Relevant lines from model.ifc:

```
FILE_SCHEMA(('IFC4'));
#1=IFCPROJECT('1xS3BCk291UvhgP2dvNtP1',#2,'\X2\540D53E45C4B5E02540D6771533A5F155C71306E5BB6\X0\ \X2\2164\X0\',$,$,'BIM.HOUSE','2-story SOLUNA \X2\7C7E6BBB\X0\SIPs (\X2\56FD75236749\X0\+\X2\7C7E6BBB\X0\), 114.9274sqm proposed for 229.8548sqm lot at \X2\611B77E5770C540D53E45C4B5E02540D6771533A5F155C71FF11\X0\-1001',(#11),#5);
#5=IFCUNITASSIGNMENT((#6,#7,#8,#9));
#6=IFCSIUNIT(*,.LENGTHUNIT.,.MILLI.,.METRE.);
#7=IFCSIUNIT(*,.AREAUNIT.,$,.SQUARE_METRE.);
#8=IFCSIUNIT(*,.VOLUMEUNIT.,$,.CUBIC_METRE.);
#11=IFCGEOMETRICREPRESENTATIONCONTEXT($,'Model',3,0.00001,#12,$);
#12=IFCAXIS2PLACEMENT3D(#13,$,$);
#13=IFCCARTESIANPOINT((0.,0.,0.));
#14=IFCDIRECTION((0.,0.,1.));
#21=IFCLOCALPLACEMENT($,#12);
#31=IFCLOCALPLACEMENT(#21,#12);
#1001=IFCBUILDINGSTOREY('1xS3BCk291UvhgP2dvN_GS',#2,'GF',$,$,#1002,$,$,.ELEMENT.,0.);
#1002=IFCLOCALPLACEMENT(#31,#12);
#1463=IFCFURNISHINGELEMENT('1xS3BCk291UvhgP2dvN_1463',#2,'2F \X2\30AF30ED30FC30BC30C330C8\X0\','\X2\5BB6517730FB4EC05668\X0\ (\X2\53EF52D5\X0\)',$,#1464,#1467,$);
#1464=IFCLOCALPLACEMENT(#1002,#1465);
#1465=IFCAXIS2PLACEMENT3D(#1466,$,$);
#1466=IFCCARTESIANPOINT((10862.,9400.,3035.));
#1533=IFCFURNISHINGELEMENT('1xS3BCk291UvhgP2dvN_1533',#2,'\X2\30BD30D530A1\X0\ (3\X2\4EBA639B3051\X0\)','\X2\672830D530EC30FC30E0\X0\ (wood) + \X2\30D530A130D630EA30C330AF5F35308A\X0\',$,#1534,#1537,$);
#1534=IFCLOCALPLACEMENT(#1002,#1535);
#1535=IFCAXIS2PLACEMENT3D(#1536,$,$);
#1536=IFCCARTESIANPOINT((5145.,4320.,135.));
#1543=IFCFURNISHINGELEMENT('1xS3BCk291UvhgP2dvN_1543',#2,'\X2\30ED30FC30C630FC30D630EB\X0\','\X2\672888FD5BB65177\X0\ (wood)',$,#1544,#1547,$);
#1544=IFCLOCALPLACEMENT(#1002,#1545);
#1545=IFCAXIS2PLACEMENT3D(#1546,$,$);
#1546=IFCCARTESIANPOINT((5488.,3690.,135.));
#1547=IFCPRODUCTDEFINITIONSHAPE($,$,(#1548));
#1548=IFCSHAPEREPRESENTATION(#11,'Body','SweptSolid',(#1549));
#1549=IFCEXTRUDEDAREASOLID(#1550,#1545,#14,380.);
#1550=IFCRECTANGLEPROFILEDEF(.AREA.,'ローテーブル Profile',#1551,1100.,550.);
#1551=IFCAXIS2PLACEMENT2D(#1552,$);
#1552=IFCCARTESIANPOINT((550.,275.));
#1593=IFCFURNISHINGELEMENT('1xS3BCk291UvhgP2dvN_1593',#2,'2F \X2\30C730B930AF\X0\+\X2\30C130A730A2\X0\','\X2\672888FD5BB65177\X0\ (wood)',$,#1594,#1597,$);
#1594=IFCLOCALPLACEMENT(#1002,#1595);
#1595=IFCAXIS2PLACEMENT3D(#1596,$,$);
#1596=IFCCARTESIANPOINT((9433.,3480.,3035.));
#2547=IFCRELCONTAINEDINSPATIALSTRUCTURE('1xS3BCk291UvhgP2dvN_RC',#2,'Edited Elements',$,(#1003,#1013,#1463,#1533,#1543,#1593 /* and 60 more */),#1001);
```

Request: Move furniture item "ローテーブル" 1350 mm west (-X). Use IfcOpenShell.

```python
import ifcopenshell
import ifcopenshell.api.geometry
import ifcopenshell.util.placement

model = ifcopenshell.open("model.ifc")

item = model.by_guid("1xS3BCk291UvhgP2dvN_1543")
matrix = ifcopenshell.util.placement.get_local_placement(item.ObjectPlacement)
matrix[0, 3] -= 1350.0
ifcopenshell.api.geometry.edit_object_placement(model, product=item, matrix=matrix, is_si=False)

print(ifcopenshell.util.placement.get_local_placement(item.ObjectPlacement).round(3) + 0.0)

model.write("model_rev.ifc")
```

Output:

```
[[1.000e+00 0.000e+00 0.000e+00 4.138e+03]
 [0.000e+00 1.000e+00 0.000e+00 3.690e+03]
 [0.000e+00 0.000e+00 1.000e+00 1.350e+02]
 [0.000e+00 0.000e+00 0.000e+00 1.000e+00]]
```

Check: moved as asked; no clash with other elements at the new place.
